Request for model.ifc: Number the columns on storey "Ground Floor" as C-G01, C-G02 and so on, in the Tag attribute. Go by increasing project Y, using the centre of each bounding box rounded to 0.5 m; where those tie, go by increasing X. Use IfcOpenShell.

First a look at what the model holds.

```python
import ifcopenshell
import ifcopenshell.util.element
import ifcopenshell.util.placement

model = ifcopenshell.open("model.ifc")
print(model.schema)
storey = next(s for s in model.by_type("IfcBuildingStorey") if s.Name == "Ground Floor")
columns = [e for e in ifcopenshell.util.element.get_decomposition(storey) if e.is_a("IfcColumn")]
for e in sorted(columns, key=lambda e: e.id()):
    origin = ifcopenshell.util.placement.get_local_placement(e.ObjectPlacement)[:3, 3]
    print(e.id(), e.Tag, e.Name, origin.round(2) + 0.0, sep=" | ")
```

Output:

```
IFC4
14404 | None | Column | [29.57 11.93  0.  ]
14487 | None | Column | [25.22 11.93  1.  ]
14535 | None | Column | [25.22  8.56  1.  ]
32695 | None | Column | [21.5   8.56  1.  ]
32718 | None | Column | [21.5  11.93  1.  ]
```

```python
import ifcopenshell
import ifcopenshell.geom
import ifcopenshell.util.element
import ifcopenshell.util.shape

model = ifcopenshell.open("model.ifc")
settings = ifcopenshell.geom.settings()
settings.set("use-world-coords", True)


def centre(element):
    shape = ifcopenshell.geom.create_shape(settings, element)
    return ifcopenshell.util.shape.get_bbox_centroid(shape.geometry)


storey = next(s for s in model.by_type("IfcBuildingStorey") if s.Name == "Ground Floor")
columns = [e for e in ifcopenshell.util.element.get_decomposition(storey) if e.is_a("IfcColumn")]

# Insertion points can sit at a corner or the storey origin, so sort by the geometry (in metres).
centres = {e: centre(e) for e in columns}
columns.sort(key=lambda e: (round(centres[e][1] / 0.5), centres[e][0]))

for i, e in enumerate(columns, start=1):
    number = f"C-G{i:02d}"
    e.Tag = number
    print(e.id(), number)

model.write("model_v2.ifc")
```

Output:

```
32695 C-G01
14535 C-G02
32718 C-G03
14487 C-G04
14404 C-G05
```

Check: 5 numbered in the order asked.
